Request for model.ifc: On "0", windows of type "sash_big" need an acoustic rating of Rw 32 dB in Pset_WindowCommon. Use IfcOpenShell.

First a look at what the model holds.

```python
import ifcopenshell
import ifcopenshell.util.element

model = ifcopenshell.open("model.ifc")
print(model.schema)
storey = next(s for s in model.by_type("IfcBuildingStorey") if s.Name == "0")
windows = [e for e in ifcopenshell.util.element.get_decomposition(storey) if e.is_a("IfcWindow")]
seen = {}
for e in windows:
    element_type = ifcopenshell.util.element.get_type(e)
    key = (element_type.Name if element_type != e and element_type else None, ifcopenshell.util.element.get_pset(e, "Pset_WindowCommon", "AcousticRating"))
    seen[key] = seen.get(key, 0) + 1
for (name, value), count in sorted(seen.items(), key=str):
    print(count, "x", name, "|", value)
```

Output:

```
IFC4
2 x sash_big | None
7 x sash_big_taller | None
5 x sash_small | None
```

```python
import ifcopenshell
import ifcopenshell.api.pset
import ifcopenshell.util.element

model = ifcopenshell.open("model.ifc")

storey = next(s for s in model.by_type("IfcBuildingStorey") if s.Name == "0")
windows = [e for e in ifcopenshell.util.element.get_decomposition(storey) if e.is_a("IfcWindow")]

count = 0
for e in windows:
    element_type = ifcopenshell.util.element.get_type(e)
    if element_type in (None, e) or element_type.Name != "sash_big":
        continue
    # add_pset returns the element's existing set when there is one.
    pset = ifcopenshell.api.pset.add_pset(model, product=e, name="Pset_WindowCommon")
    ifcopenshell.api.pset.edit_pset(model, pset=pset, properties={"AcousticRating": "Rw 32 dB"})
    count += 1

print(count, "windows updated")

model.write("model_updated.ifc")
```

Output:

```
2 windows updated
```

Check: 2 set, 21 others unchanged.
